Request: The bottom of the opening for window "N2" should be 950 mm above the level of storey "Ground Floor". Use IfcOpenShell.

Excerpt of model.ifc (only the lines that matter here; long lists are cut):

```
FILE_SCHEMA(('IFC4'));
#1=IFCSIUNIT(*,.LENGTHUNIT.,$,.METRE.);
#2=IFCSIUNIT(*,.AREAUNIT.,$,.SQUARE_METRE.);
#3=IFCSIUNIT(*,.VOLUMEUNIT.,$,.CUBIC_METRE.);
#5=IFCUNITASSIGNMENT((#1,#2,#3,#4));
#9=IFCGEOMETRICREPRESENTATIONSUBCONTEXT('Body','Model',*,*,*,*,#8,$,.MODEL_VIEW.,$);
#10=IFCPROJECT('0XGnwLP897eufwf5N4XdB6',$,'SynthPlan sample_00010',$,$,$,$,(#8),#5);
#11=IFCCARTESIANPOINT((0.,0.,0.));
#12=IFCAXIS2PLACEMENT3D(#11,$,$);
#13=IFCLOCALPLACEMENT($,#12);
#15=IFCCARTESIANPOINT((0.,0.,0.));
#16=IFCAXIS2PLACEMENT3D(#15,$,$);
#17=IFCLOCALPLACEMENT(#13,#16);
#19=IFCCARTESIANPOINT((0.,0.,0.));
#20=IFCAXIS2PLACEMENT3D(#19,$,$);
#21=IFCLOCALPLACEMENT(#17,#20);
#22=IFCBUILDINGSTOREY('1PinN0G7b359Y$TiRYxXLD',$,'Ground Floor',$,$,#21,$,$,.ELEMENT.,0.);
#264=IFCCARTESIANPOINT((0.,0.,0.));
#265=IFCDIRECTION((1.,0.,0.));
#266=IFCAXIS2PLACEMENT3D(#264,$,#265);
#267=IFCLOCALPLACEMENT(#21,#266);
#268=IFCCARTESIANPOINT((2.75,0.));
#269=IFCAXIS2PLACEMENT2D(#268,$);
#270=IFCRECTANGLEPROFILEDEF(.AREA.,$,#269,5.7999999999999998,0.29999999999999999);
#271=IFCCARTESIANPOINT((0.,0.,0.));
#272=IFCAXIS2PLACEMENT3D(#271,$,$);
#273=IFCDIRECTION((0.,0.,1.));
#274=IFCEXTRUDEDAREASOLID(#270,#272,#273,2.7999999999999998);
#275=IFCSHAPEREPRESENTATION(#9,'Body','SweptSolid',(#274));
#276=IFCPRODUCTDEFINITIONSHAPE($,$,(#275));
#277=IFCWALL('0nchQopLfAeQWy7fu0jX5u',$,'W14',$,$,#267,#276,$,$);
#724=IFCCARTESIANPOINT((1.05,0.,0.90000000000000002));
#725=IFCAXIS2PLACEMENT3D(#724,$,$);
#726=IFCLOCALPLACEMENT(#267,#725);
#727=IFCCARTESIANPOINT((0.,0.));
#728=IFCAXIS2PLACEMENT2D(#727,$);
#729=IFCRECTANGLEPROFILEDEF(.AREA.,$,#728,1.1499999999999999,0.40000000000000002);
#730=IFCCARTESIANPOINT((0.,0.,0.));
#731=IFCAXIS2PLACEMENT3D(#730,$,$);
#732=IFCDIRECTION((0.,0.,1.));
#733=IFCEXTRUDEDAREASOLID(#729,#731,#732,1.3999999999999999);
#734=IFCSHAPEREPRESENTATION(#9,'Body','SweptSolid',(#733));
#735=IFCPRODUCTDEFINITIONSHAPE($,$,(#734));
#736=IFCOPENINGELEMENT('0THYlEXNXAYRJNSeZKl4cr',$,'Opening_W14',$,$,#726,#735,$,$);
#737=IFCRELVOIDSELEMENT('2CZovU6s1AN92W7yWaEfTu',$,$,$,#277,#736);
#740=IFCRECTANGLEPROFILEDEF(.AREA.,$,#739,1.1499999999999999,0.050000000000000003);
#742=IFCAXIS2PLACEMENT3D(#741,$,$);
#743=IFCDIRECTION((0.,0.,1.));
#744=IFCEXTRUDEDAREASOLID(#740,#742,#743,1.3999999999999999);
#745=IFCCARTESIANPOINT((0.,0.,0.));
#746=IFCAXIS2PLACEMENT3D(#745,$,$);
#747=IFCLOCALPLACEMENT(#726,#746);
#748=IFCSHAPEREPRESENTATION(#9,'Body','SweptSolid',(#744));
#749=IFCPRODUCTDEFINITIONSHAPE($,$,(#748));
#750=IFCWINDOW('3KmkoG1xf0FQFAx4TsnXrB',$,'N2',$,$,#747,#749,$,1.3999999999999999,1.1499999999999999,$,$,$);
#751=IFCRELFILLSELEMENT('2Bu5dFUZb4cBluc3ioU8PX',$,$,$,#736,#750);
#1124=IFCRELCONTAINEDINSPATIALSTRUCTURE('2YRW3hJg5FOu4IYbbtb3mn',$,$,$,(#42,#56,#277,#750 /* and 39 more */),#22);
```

```python
import numpy as np
import ifcopenshell
import ifcopenshell.api.geometry
import ifcopenshell.geom
import ifcopenshell.util.element
import ifcopenshell.util.placement
import ifcopenshell.util.shape
import ifcopenshell.util.unit

model = ifcopenshell.open("model.ifc")
unit_scale = ifcopenshell.util.unit.calculate_unit_scale(model)

window = model.by_id(750)
opening = window.FillsVoids[0].RelatingOpeningElement
storey = ifcopenshell.util.element.get_container(window, ifc_class="IfcBuildingStorey")
level = ifcopenshell.util.placement.get_local_placement(storey.ObjectPlacement)[2, 3]

# The opening's origin need not be at the sill, so measure its lowest point.
shape = ifcopenshell.geom.create_shape(ifcopenshell.geom.settings(), opening)
bottom = ifcopenshell.util.shape.get_shape_bottom_elevation(shape, shape.geometry) / unit_scale
dz = level + 0.95 / unit_scale - bottom

shift = np.array([0.0, 0.0, dz])
# The window is placed relative to its opening, so it follows when the opening moves.
matrix = ifcopenshell.util.placement.get_local_placement(opening.ObjectPlacement)
matrix[:3, 3] += shift
ifcopenshell.api.geometry.edit_object_placement(
    model, product=opening, matrix=matrix, is_si=False, should_transform_children=True
)

print(f"moved by {dz * unit_scale:+.3f} m")

model.write("model_edited.ifc")
```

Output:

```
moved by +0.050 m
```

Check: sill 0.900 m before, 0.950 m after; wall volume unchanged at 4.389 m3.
